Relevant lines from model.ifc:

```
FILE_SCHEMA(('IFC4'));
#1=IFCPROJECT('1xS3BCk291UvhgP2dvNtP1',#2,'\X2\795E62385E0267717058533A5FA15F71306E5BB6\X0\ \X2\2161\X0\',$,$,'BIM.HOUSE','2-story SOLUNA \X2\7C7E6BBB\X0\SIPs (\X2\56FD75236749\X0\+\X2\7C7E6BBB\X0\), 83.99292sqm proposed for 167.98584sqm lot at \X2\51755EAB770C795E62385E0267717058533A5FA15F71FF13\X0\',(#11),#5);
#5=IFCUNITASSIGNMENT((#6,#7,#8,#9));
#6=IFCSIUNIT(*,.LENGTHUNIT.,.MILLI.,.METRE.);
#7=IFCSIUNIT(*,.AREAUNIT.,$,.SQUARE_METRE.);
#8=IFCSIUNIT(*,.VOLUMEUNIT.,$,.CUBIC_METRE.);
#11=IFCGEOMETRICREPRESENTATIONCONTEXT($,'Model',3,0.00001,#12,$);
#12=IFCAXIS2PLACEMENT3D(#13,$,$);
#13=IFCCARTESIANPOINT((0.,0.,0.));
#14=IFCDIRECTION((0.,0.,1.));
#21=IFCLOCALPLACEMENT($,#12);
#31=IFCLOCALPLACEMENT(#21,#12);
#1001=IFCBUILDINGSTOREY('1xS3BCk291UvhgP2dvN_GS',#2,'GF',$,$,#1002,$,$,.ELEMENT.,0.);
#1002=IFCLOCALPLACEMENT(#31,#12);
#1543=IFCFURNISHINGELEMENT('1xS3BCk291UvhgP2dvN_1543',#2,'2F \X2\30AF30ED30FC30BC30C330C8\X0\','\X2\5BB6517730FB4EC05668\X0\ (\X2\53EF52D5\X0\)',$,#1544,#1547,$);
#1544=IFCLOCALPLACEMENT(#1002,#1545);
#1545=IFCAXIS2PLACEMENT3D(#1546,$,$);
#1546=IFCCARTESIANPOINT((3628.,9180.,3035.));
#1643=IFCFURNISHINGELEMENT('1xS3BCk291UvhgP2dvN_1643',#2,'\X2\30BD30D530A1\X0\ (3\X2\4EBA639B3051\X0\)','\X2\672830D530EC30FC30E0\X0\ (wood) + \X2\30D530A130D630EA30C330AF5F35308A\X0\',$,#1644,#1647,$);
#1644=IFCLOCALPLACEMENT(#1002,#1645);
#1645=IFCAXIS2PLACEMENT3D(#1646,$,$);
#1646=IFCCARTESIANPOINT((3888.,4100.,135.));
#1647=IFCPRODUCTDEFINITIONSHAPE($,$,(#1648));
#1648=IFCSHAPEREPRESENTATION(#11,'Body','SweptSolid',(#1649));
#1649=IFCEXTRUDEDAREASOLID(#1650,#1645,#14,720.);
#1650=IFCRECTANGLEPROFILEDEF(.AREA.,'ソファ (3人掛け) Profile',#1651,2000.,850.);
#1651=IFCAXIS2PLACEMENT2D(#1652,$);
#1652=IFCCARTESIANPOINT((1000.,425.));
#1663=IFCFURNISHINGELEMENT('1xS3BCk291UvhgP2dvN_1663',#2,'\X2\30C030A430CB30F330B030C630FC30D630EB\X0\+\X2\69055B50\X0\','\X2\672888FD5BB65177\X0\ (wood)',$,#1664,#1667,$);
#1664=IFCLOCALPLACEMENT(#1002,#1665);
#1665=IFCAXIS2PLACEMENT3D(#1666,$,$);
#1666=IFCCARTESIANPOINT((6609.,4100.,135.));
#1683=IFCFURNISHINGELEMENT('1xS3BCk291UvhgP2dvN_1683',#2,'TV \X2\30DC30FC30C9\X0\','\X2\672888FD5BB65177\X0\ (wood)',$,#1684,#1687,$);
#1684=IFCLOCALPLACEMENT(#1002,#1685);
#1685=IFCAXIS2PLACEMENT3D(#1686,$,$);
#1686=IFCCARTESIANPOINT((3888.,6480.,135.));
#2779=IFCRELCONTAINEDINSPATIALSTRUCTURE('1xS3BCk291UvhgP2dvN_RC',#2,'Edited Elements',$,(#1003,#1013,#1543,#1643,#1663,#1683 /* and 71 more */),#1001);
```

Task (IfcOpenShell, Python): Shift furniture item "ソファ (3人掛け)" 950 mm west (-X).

```python
import ifcopenshell
import ifcopenshell.api.geometry
import ifcopenshell.util.placement

model = ifcopenshell.open("model.ifc")

item = model.by_id(1643)
matrix = ifcopenshell.util.placement.get_local_placement(item.ObjectPlacement)
matrix[0, 3] -= 950.0
ifcopenshell.api.geometry.edit_object_placement(model, product=item, matrix=matrix, is_si=False)

print(ifcopenshell.util.placement.get_local_placement(item.ObjectPlacement).round(3) + 0.0)

model.write("model_v2.ifc")
```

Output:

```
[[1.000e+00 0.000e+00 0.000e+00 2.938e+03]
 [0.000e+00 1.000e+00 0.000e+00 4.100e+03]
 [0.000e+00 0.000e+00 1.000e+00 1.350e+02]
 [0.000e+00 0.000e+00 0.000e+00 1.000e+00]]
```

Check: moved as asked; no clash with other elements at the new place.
